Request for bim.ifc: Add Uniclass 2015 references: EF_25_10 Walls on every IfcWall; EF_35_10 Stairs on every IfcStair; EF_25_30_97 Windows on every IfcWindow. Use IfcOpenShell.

First a look at what the model holds.

```python
import ifcopenshell

model = ifcopenshell.open("bim.ifc")
print(model.schema)
print("classifications:", [c.Name for c in model.by_type("IfcClassification")])
for ifc_class in ("IfcDoor", "IfcRoof", "IfcStair", "IfcWall", "IfcWindow"):
    print(ifc_class, len(model.by_type(ifc_class)))
```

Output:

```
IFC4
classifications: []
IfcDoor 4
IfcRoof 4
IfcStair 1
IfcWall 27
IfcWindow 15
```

```python
import ifcopenshell
import ifcopenshell.api.classification

model = ifcopenshell.open("bim.ifc")

system = ifcopenshell.api.classification.add_classification(model, classification="Uniclass 2015")

codes = {
    "IfcWall": ("EF_25_10", "Walls"),
    "IfcStair": ("EF_35_10", "Stairs"),
    "IfcWindow": ("EF_25_30_97", "Windows"),
}
for ifc_class, (code, name) in codes.items():
    products = model.by_type(ifc_class)
    ifcopenshell.api.classification.add_reference(
        model, products=products, classification=system, identification=code, name=name
    )
    print(code, len(products))

model.write("bim_edited.ifc")
```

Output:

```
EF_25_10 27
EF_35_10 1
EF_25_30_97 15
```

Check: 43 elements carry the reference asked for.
